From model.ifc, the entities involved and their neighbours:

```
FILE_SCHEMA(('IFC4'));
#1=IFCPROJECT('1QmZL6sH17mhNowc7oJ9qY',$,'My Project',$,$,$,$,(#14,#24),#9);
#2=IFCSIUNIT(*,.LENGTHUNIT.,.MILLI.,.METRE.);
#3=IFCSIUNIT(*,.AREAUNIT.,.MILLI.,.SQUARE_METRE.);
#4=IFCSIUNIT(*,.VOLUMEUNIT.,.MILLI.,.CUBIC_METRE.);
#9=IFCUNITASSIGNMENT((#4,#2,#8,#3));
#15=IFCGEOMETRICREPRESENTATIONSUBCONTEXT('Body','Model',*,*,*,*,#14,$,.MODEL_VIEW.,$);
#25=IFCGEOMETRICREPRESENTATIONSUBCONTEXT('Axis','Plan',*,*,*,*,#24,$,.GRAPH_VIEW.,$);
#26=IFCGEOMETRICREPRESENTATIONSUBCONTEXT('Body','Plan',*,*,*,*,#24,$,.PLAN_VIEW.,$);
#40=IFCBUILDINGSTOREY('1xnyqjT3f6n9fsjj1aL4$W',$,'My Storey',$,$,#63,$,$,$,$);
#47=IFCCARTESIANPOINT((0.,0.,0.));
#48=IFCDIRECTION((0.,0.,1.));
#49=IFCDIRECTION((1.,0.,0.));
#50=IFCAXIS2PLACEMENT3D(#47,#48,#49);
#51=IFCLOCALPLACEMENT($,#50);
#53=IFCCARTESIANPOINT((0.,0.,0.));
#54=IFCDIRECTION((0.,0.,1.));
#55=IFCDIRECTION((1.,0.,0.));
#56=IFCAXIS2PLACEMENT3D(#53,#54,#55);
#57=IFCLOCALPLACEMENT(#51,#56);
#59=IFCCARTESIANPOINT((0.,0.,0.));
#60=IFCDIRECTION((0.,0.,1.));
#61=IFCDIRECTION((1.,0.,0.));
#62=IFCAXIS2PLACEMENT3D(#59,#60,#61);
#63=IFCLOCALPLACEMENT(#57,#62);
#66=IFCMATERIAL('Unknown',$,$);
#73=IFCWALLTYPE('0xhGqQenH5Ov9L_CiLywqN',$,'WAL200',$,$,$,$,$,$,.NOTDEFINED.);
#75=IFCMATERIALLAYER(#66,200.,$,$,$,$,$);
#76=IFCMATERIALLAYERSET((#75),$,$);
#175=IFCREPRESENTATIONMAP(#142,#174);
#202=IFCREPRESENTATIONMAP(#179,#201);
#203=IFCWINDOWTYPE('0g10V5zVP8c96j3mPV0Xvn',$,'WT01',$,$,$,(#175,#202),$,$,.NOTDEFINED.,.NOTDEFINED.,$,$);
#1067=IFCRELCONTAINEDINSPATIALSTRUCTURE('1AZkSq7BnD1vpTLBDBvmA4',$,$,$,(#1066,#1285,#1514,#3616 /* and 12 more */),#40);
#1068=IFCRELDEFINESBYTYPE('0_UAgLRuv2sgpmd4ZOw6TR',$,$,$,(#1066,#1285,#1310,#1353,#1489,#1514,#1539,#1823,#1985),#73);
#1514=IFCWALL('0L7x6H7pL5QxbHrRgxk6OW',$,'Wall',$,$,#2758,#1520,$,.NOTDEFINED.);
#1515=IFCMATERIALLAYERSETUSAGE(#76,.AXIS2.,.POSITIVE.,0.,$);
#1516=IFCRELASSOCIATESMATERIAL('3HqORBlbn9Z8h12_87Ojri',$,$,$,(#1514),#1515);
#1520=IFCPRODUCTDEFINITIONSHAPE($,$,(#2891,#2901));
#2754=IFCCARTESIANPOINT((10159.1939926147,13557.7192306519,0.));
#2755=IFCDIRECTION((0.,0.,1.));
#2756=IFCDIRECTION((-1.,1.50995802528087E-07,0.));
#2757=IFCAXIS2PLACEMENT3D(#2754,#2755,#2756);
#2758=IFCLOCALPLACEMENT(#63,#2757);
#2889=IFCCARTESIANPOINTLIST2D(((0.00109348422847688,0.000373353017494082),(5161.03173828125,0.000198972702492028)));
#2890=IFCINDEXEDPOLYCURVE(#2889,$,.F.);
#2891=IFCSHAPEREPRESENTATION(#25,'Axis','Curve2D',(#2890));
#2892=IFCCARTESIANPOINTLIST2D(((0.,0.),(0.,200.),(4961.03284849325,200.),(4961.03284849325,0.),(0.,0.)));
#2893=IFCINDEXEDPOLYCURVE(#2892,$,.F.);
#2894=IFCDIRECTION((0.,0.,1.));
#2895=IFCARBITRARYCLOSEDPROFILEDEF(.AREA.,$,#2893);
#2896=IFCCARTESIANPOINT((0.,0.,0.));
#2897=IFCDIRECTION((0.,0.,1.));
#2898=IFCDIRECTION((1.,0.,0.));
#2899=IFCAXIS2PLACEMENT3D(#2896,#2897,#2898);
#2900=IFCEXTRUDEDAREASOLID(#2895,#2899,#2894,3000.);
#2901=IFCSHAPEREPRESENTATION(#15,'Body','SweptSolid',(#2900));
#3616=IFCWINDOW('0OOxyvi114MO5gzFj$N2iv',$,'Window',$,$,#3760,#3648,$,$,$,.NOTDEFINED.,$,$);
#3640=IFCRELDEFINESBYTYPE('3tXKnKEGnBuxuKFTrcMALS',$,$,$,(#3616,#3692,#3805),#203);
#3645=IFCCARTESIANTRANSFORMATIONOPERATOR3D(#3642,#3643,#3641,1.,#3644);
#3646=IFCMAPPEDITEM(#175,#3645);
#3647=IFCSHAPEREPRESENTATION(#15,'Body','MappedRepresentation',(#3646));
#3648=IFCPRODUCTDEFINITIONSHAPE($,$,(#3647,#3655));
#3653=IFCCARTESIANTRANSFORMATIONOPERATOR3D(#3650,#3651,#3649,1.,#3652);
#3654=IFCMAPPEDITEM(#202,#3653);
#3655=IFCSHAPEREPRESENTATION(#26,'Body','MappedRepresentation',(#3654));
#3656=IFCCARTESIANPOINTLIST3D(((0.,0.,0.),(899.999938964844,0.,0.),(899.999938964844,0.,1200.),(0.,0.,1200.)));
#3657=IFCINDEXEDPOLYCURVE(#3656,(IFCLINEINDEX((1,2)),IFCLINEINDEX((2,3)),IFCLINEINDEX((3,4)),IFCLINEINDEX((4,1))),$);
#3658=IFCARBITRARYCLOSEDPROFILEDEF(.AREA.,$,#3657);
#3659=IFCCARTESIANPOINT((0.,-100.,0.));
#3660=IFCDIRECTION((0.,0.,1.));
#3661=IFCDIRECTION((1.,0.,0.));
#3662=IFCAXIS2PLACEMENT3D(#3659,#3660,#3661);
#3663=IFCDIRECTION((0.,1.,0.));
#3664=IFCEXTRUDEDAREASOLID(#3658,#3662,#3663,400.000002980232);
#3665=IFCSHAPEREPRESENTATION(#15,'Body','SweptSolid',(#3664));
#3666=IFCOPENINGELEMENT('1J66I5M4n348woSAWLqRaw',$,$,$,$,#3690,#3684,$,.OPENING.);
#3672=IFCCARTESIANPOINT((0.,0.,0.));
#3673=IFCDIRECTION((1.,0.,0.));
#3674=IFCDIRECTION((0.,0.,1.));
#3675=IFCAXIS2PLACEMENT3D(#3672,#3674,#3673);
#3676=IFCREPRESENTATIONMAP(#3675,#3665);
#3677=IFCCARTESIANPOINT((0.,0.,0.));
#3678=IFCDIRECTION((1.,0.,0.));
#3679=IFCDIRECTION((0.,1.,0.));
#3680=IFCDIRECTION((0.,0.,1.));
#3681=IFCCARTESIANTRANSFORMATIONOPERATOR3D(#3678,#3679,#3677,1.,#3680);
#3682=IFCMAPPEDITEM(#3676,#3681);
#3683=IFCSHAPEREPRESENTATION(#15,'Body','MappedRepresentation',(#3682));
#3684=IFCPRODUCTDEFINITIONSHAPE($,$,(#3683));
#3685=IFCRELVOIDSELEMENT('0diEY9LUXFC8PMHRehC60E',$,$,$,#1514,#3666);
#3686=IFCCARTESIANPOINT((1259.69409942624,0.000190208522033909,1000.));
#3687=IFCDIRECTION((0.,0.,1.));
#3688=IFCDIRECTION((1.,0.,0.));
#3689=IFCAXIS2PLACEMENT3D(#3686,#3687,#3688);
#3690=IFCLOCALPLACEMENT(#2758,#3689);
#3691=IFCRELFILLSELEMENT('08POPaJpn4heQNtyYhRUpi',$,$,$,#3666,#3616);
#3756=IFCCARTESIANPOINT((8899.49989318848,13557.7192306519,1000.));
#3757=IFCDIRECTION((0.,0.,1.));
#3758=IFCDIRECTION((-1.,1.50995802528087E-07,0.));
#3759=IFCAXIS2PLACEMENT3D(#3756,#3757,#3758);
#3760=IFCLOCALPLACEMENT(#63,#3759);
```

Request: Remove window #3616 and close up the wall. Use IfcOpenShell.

```python
import ifcopenshell
import ifcopenshell.api.feature
import ifcopenshell.api.root
import ifcopenshell.geom
import ifcopenshell.util.shape

model = ifcopenshell.open("model.ifc")
settings = ifcopenshell.geom.settings()


def volume(element):
    """Net volume in cubic metres, openings subtracted."""
    shape = ifcopenshell.geom.create_shape(settings, element)
    return ifcopenshell.util.shape.get_volume(shape.geometry)


window = model.by_guid("0OOxyvi114MO5gzFj$N2iv")
opening = window.FillsVoids[0].RelatingOpeningElement
wall = opening.VoidsElements[0].RelatingBuildingElement
before = volume(wall)

ifcopenshell.api.root.remove_product(model, product=window)
ifcopenshell.api.feature.remove_feature(model, feature=opening)

after = volume(wall)

print(f"wall volume {before:.3f} -> {after:.3f} m3")

model.write("model_rev.ifc")
```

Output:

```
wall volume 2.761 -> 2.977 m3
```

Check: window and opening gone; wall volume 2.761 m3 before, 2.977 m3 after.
